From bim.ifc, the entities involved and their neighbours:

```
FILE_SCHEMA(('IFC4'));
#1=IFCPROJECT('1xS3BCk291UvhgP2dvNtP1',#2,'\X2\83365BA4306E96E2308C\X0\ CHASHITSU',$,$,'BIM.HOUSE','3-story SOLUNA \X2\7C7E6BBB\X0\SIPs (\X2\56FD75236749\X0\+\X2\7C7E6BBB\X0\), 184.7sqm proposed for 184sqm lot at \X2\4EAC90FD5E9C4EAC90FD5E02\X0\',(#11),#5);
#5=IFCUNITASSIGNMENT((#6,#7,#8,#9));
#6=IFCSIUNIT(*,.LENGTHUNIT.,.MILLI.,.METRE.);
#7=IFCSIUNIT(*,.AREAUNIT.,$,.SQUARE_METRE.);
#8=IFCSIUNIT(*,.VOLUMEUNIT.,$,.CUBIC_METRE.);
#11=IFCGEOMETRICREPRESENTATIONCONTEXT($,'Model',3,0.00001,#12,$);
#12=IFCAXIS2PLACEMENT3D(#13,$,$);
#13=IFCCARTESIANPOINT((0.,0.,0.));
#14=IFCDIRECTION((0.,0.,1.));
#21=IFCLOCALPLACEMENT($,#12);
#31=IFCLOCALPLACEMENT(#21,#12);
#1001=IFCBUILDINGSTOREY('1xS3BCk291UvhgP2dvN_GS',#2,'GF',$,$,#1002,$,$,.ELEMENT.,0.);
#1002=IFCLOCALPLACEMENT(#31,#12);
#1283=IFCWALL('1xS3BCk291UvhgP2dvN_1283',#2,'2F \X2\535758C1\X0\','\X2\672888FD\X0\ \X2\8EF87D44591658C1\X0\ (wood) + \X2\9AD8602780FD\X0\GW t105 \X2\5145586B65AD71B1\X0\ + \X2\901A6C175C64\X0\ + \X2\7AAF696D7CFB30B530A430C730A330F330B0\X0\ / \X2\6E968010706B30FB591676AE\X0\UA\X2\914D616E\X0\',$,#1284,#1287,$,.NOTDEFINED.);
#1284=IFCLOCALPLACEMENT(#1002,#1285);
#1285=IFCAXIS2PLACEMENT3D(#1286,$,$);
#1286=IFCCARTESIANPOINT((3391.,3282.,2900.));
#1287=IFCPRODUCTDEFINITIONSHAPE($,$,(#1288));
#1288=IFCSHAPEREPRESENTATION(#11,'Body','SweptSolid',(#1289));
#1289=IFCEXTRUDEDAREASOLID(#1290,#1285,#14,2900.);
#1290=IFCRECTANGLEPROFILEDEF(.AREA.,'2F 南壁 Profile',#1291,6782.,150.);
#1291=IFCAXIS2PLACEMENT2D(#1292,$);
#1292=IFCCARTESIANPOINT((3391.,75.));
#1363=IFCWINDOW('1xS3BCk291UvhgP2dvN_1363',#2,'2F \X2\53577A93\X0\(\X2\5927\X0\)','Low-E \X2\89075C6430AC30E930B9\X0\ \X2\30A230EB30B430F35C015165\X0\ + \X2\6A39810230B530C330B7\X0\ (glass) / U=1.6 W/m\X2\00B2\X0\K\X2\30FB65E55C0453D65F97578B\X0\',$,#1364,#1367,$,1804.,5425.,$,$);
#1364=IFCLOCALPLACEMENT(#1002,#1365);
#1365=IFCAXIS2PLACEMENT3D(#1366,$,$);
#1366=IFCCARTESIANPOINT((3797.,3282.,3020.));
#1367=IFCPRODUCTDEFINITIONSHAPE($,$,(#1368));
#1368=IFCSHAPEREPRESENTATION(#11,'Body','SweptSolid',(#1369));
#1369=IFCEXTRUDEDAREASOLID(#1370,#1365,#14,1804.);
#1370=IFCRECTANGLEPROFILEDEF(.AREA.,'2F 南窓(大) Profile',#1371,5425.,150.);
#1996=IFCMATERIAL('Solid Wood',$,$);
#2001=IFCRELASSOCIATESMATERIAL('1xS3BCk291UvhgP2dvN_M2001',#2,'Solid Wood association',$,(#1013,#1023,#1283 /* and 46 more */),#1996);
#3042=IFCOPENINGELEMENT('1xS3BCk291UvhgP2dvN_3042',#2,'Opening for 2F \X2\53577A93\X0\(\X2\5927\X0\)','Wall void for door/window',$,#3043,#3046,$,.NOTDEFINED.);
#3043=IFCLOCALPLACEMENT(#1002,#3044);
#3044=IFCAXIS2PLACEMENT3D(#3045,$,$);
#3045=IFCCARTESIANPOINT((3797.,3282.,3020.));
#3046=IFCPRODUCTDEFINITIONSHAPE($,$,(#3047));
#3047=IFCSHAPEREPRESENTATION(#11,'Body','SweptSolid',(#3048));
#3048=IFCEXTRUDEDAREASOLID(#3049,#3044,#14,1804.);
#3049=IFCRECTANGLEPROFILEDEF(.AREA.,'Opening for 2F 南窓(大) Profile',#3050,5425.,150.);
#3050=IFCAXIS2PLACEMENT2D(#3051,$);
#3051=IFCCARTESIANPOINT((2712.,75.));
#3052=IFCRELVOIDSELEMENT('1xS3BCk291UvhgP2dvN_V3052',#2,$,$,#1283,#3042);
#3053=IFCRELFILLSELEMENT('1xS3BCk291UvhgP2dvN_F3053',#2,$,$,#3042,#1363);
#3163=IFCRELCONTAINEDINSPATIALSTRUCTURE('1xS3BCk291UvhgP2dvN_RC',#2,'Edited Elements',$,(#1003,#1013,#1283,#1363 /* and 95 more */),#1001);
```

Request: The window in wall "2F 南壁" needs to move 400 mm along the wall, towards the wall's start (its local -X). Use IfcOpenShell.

```python
import ifcopenshell
import ifcopenshell.api.geometry
import ifcopenshell.util.placement

model = ifcopenshell.open("bim.ifc")

window = model.by_guid("1xS3BCk291UvhgP2dvN_1363")
opening = window.FillsVoids[0].RelatingOpeningElement
wall = opening.VoidsElements[0].RelatingBuildingElement

wall_matrix = ifcopenshell.util.placement.get_local_placement(wall.ObjectPlacement)
shift = wall_matrix[:3, 0] * -400.0
before = ifcopenshell.util.placement.get_local_placement(window.ObjectPlacement)[:3, 3].copy()

# The window is not placed relative to its opening, so move both.
for product in (opening, window):
    matrix = ifcopenshell.util.placement.get_local_placement(product.ObjectPlacement)
    matrix[:3, 3] += shift
    ifcopenshell.api.geometry.edit_object_placement(model, product=product, matrix=matrix, is_si=False)

after = ifcopenshell.util.placement.get_local_placement(window.ObjectPlacement)[:3, 3]
print("window moved by", (after - before).round(3) + 0.0)

model.write("bim_v2.ifc")
```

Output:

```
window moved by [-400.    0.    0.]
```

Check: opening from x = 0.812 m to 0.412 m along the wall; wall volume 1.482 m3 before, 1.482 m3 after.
